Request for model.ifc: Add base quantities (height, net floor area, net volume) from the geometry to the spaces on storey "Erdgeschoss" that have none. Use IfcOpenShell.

First a look at what the model holds.

```python
import ifcopenshell
import ifcopenshell.util.element
import ifcopenshell.util.unit

model = ifcopenshell.open("model.ifc")
print(model.schema)
for unit_type in ("LENGTHUNIT", "AREAUNIT", "VOLUMEUNIT"):
    print(unit_type, ifcopenshell.util.unit.calculate_unit_scale(model, unit_type))
storey = next(s for s in model.by_type("IfcBuildingStorey") if s.Name == "Erdgeschoss")
spaces = [e for e in ifcopenshell.util.element.get_decomposition(storey) if e.is_a("IfcSpace")]
for e in sorted(spaces, key=lambda e: e.id()):
    print(e.id(), e.is_a(), e.Name, list(ifcopenshell.util.element.get_psets(e, qtos_only=True)), sep=" | ")
```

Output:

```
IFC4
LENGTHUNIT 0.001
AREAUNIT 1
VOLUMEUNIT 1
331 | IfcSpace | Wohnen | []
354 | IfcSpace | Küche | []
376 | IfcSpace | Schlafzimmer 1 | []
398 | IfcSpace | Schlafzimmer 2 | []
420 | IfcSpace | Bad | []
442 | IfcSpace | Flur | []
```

```python
import ifcopenshell
import ifcopenshell.api.pset
import ifcopenshell.geom
import ifcopenshell.util.element
import ifcopenshell.util.shape
import ifcopenshell.util.unit

model = ifcopenshell.open("model.ifc")
unit_scale = ifcopenshell.util.unit.calculate_unit_scale(model)
area_scale = ifcopenshell.util.unit.calculate_unit_scale(model, "AREAUNIT")
volume_scale = ifcopenshell.util.unit.calculate_unit_scale(model, "VOLUMEUNIT")
settings = ifcopenshell.geom.settings()

storey = next(s for s in model.by_type("IfcBuildingStorey") if s.Name == "Erdgeschoss")
spaces = [e for e in ifcopenshell.util.element.get_decomposition(storey) if e.is_a("IfcSpace")]

for e in sorted(spaces, key=lambda e: e.id()):
    if ifcopenshell.util.element.get_psets(e, qtos_only=True, should_inherit=False):
        continue
    # Geometry comes back in metres, in the element's own axes.
    shape = ifcopenshell.geom.create_shape(settings, e)
    values = {
        "Height": ifcopenshell.util.shape.get_z(shape.geometry) / unit_scale,
        "NetFloorArea": ifcopenshell.util.shape.get_footprint_area(shape.geometry) / area_scale,
        "NetVolume": ifcopenshell.util.shape.get_volume(shape.geometry) / volume_scale,
    }
    qto = ifcopenshell.api.pset.add_qto(model, product=e, name="Qto_SpaceBaseQuantities")
    ifcopenshell.api.pset.edit_qto(model, qto=qto, properties=values)
    print(e.id(), {k: round(v, 3) for k, v in values.items()})

model.write("model_rev.ifc")
```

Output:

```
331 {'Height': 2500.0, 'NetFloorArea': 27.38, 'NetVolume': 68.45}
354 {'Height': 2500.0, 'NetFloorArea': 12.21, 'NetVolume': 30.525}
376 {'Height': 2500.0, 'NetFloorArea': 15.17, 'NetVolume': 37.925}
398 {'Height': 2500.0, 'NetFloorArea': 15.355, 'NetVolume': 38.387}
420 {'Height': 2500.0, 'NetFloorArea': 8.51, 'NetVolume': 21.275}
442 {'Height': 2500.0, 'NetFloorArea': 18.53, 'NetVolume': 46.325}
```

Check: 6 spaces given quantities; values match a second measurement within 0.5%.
